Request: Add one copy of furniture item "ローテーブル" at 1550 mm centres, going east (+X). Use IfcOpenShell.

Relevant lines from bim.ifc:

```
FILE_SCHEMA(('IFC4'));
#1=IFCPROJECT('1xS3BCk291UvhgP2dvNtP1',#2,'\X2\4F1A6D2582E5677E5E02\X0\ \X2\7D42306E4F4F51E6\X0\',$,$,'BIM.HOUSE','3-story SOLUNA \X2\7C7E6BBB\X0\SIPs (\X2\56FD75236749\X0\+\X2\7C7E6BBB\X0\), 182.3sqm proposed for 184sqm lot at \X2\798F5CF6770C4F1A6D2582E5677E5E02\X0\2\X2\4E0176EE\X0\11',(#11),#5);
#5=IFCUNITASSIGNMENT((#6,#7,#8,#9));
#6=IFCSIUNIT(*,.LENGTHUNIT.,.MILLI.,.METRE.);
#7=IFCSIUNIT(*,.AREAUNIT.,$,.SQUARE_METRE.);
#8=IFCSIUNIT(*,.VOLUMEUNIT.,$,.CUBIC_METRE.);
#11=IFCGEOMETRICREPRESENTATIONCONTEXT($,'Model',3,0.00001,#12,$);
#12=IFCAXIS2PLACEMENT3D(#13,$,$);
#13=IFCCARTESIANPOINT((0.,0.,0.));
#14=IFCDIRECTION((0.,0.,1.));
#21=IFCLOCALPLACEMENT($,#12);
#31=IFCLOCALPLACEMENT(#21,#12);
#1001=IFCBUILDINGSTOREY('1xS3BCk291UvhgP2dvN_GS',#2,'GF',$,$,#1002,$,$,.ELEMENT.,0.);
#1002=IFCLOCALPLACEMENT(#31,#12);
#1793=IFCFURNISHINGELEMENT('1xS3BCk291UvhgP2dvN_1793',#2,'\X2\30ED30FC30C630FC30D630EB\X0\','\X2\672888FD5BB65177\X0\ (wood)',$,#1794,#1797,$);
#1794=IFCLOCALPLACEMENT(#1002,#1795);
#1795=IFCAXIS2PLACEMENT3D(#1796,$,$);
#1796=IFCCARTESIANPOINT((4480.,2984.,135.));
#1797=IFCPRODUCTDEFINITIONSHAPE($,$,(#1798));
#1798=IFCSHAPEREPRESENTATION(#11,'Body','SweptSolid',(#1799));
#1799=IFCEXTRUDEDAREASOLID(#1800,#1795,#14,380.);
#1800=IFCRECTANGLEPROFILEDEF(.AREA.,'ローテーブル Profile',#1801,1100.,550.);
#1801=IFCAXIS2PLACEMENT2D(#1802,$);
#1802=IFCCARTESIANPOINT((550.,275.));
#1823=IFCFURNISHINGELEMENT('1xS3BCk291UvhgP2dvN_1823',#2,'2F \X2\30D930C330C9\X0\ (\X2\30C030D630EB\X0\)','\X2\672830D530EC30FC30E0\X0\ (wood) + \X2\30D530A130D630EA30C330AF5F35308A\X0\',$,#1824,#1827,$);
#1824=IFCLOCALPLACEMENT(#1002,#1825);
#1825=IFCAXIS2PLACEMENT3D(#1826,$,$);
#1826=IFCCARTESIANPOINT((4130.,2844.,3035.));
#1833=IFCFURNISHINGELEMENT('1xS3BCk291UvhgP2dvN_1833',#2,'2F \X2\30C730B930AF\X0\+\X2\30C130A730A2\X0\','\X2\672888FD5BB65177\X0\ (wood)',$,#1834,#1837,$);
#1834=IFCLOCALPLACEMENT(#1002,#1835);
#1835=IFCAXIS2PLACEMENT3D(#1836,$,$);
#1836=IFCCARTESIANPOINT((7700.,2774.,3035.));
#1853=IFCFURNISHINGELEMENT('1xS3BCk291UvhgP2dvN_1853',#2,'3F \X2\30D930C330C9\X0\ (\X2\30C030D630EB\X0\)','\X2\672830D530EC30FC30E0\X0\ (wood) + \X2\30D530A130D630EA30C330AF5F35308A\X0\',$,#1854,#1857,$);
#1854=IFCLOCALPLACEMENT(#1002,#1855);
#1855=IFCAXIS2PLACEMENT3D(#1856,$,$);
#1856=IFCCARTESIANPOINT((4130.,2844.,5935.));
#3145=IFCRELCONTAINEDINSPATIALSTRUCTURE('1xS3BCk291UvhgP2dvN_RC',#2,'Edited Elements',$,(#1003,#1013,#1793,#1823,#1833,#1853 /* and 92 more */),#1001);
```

```python
import numpy as np
import ifcopenshell
import ifcopenshell.api.geometry
import ifcopenshell.api.root
import ifcopenshell.util.element
import ifcopenshell.util.placement
import ifcopenshell.util.unit

model = ifcopenshell.open("bim.ifc")
unit_scale = ifcopenshell.util.unit.calculate_unit_scale(model)


def reuse_history(source, copy):
    """copy_class also copies each property set's owner history, people and application; keep the originals."""
    for rel in copy.IsDefinedBy:
        if rel.is_a("IfcRelDefinesByProperties") and (history := rel.RelatingPropertyDefinition.OwnerHistory):
            rel.RelatingPropertyDefinition.OwnerHistory = source.OwnerHistory
            ifcopenshell.util.element.remove_deep2(model, history)


source = model.by_guid("1xS3BCk291UvhgP2dvN_1793")
base = ifcopenshell.util.placement.get_local_placement(source.ObjectPlacement)
step = np.array([1.0, 0.0, 0.0]) * 1.55 / unit_scale

for i in range(1, 2):
    copy = ifcopenshell.api.root.copy_class(model, product=source)
    copy.Representation = ifcopenshell.util.element.copy_deep(
        model, source.Representation, exclude=["IfcGeometricRepresentationContext", "IfcRepresentationMap"]
    )
    reuse_history(source, copy)
    matrix = base.copy()
    matrix[:3, 3] += i * step
    print("added at", matrix[:3, 3].round(3) + 0.0)
    ifcopenshell.api.geometry.edit_object_placement(model, product=copy, matrix=matrix, is_si=False)

model.write("bim_edited.ifc")
```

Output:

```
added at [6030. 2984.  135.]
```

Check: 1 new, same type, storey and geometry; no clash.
